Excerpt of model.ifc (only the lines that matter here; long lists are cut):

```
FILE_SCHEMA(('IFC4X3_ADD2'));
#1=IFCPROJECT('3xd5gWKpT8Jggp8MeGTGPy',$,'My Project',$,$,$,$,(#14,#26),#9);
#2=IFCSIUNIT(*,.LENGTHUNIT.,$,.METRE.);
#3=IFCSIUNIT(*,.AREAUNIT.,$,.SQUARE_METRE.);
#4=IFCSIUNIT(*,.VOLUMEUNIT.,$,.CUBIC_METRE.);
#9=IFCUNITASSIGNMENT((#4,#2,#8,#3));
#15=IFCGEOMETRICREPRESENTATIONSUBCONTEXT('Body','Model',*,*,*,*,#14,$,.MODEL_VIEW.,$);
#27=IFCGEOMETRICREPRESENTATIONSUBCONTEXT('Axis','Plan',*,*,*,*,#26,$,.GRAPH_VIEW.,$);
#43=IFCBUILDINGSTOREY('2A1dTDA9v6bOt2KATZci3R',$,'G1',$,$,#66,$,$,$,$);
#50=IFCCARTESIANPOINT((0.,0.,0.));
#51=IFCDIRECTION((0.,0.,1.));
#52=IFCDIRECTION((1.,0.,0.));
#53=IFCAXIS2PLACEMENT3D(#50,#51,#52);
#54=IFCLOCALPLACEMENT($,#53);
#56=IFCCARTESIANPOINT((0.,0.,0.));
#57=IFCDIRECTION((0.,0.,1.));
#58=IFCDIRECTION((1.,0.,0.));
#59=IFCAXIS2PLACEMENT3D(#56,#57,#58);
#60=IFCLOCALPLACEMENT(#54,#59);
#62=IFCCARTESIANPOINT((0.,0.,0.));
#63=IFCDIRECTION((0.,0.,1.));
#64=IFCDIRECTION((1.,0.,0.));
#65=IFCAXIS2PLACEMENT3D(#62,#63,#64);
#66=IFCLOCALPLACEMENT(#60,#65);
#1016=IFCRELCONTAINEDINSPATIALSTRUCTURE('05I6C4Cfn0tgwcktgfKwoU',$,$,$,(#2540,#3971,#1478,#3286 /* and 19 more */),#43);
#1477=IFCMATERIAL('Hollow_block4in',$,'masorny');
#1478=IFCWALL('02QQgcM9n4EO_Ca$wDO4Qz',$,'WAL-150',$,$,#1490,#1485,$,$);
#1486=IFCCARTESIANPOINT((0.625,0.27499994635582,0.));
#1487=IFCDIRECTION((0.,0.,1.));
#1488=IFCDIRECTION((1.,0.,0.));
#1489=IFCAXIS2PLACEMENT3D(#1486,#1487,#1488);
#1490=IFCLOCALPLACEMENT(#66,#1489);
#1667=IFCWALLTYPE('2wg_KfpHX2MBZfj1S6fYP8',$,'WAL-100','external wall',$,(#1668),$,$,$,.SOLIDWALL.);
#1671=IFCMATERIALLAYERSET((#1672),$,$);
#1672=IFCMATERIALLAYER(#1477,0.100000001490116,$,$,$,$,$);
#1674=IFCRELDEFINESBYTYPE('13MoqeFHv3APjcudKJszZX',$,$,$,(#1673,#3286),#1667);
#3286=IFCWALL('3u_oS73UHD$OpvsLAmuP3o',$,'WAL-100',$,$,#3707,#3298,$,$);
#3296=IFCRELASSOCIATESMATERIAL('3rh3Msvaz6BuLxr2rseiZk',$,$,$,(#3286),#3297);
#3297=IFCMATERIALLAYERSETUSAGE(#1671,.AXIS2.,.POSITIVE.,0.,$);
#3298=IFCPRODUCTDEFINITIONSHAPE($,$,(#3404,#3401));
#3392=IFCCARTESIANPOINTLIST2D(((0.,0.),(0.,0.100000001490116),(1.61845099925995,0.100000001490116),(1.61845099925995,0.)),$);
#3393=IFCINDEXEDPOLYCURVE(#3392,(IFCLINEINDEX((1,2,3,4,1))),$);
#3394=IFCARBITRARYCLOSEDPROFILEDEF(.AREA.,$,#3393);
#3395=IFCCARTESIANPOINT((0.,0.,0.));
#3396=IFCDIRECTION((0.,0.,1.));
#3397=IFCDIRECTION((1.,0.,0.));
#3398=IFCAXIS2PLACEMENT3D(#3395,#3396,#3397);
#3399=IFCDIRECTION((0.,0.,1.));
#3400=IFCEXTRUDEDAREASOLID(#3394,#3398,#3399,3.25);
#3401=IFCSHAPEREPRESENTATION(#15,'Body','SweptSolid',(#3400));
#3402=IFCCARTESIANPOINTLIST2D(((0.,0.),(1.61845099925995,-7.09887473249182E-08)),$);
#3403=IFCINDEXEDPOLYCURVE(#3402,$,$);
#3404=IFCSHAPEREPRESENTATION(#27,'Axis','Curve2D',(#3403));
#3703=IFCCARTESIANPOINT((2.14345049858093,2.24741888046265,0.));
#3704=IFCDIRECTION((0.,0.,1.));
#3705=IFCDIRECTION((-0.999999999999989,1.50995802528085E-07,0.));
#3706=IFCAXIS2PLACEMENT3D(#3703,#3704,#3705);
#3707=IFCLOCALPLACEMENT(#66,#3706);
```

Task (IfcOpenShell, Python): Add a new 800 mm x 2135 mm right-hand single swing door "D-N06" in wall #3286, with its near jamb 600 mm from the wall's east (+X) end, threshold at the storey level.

```python
import numpy as np
import ifcopenshell
import ifcopenshell.api.feature
import ifcopenshell.api.geometry
import ifcopenshell.api.root
import ifcopenshell.api.spatial
import ifcopenshell.geom
import ifcopenshell.util.element
import ifcopenshell.util.placement
import ifcopenshell.util.representation
import ifcopenshell.util.shape
import ifcopenshell.util.unit

model = ifcopenshell.open("model.ifc")
unit_scale = ifcopenshell.util.unit.calculate_unit_scale(model)
settings = ifcopenshell.geom.settings()


def volume(element):
    """Net volume in cubic metres, openings subtracted."""
    shape = ifcopenshell.geom.create_shape(settings, element)
    return ifcopenshell.util.shape.get_volume(shape.geometry)


wall = model.by_guid("3u_oS73UHD$OpvsLAmuP3o")
storey = ifcopenshell.util.element.get_container(wall, ifc_class="IfcBuildingStorey")
context = ifcopenshell.util.representation.get_context(model, "Model", "Body", "MODEL_VIEW")
before = volume(wall)

width, height, from_end, sill = 0.8, 2.135, 0.6, 0.0  # metres

# The wall runs along its own X axis, and the end named is its -X end.
wall_shape = ifcopenshell.geom.create_shape(settings, wall)
x, y, z = ifcopenshell.util.shape.get_vertices(wall_shape.geometry).T
start = x.min() + from_end
face, thickness = float(y.min()), float(y.max() - y.min())
wall_matrix = ifcopenshell.util.placement.get_local_placement(wall.ObjectPlacement)
level = ifcopenshell.util.placement.get_local_placement(storey.ObjectPlacement)[2, 3]


def in_wall(x, y):
    """Placement at x, y metres in the wall's axes, at sill height."""
    matrix = wall_matrix.copy()
    matrix[:, 3] = wall_matrix @ np.array([x / unit_scale, y / unit_scale, 0.0, 1.0])
    matrix[2, 3] = level + sill / unit_scale
    return matrix


# Opening: a box that overshoots both wall faces by 50 mm.
opening = ifcopenshell.api.root.create_entity(model, ifc_class="IfcOpeningElement", predefined_type="OPENING")
box = ifcopenshell.api.geometry.add_wall_representation(
    model, context=context, length=width, height=height, thickness=thickness + 0.1
)
ifcopenshell.api.geometry.assign_representation(model, product=opening, representation=box)
ifcopenshell.api.geometry.edit_object_placement(model, product=opening, matrix=in_wall(start, face - 0.05), is_si=False)
ifcopenshell.api.feature.add_feature(model, feature=opening, element=wall)

door = ifcopenshell.api.root.create_entity(model, ifc_class="IfcDoor", name="D-N06", predefined_type="DOOR")
door.OverallWidth, door.OverallHeight = width / unit_scale, height / unit_scale
door.OperationType = "SINGLE_SWING_RIGHT"
body = ifcopenshell.api.geometry.add_door_representation(
    model,
    context=context,
    overall_width=door.OverallWidth,
    overall_height=door.OverallHeight,
    operation_type="SINGLE_SWING_RIGHT",
    lining_properties={"LiningDepth": thickness / unit_scale, "ThresholdDepth": thickness / unit_scale},
)
ifcopenshell.api.geometry.assign_representation(model, product=door, representation=body)
ifcopenshell.api.spatial.assign_container(model, products=[door], relating_structure=storey)
ifcopenshell.api.feature.add_filling(model, opening=opening, element=door)

# The lining spans the wall, so the door starts at the wall face.
ifcopenshell.api.geometry.edit_object_placement(model, product=door, matrix=in_wall(start, face), is_si=False)

after = volume(wall)

print(f"wall volume {before:.3f} -> {after:.3f} m3")

model.write("model_edited.ifc")
```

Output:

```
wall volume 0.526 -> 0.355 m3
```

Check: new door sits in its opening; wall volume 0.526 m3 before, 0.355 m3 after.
